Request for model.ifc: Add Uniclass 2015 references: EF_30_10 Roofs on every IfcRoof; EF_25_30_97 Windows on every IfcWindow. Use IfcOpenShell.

First a look at what the model holds.

```python
import ifcopenshell

model = ifcopenshell.open("model.ifc")
print(model.schema)
print("classifications:", [c.Name for c in model.by_type("IfcClassification")])
for ifc_class in ("IfcDoor", "IfcRoof", "IfcStair", "IfcWall", "IfcWindow"):
    print(ifc_class, len(model.by_type(ifc_class)))
```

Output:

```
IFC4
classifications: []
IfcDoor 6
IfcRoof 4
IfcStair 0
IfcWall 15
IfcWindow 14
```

```python
import ifcopenshell
import ifcopenshell.api.classification

model = ifcopenshell.open("model.ifc")

system = ifcopenshell.api.classification.add_classification(model, classification="Uniclass 2015")

codes = {
    "IfcRoof": ("EF_30_10", "Roofs"),
    "IfcWindow": ("EF_25_30_97", "Windows"),
}
for ifc_class, (code, name) in codes.items():
    products = model.by_type(ifc_class)
    ifcopenshell.api.classification.add_reference(
        model, products=products, classification=system, identification=code, name=name
    )
    print(code, len(products))

model.write("model_v2.ifc")
```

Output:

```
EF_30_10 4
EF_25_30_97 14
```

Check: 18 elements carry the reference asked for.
